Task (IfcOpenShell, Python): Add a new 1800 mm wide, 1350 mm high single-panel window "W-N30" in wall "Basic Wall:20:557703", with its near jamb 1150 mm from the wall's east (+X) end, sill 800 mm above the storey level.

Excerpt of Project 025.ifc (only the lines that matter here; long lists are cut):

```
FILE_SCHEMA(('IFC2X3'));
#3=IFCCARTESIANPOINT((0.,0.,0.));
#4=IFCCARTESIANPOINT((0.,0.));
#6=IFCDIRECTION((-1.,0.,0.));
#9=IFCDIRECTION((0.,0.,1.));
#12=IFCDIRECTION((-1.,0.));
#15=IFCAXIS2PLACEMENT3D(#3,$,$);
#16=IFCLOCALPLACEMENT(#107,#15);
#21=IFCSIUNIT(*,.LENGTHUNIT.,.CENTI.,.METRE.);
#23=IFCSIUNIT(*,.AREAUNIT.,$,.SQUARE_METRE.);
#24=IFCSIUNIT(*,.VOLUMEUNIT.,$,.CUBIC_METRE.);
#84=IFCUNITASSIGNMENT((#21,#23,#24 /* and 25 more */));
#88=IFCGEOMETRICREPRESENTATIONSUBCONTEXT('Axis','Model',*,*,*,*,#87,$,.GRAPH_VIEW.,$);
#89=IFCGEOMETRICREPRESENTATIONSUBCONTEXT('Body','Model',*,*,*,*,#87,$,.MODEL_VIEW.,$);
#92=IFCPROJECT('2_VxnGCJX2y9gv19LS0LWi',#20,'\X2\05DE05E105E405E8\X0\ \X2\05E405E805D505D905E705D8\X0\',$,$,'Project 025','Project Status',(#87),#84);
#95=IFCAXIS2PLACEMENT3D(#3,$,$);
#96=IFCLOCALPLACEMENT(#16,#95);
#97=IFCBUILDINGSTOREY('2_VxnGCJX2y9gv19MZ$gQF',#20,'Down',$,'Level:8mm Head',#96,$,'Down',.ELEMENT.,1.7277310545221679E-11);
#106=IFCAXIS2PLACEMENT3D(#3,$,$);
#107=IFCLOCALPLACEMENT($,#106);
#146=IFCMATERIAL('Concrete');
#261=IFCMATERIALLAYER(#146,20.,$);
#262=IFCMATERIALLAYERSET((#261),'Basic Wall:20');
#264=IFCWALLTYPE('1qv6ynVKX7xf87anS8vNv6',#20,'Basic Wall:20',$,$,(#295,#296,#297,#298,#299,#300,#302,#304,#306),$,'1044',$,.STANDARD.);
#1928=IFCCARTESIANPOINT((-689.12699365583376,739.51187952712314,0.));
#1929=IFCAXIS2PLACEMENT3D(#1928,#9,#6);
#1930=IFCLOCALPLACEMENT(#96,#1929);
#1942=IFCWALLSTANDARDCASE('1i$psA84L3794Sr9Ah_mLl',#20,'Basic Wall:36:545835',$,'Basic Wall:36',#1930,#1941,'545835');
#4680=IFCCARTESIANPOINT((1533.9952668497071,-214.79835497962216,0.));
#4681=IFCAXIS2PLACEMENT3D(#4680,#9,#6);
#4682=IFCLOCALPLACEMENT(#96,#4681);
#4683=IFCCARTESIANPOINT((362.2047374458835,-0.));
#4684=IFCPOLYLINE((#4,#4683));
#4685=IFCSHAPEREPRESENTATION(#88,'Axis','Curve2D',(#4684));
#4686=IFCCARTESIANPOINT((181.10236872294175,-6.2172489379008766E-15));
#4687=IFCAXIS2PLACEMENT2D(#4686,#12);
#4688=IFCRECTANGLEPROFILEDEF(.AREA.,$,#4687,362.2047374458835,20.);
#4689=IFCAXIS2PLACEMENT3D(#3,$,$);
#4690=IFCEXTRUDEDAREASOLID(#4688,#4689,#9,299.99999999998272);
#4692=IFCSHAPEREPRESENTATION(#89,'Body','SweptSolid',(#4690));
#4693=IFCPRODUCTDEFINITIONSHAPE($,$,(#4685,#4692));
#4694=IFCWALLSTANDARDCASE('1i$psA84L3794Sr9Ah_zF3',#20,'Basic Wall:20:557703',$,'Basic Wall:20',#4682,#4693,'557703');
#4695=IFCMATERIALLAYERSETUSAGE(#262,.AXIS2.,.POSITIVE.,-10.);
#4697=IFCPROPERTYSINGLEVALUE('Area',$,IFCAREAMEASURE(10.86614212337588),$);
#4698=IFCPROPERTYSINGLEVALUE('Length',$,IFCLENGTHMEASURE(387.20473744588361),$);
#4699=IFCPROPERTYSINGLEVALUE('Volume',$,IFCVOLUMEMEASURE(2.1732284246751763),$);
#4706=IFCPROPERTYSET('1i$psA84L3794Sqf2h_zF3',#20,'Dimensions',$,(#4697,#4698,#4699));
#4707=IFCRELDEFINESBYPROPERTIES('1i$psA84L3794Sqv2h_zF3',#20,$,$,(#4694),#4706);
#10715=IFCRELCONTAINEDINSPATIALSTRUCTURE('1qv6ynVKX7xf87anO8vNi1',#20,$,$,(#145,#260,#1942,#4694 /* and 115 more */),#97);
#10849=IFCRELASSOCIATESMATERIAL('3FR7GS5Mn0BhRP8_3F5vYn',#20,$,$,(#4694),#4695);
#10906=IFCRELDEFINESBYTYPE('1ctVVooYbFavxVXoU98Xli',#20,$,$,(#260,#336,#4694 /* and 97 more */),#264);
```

```python
import numpy as np
import ifcopenshell
import ifcopenshell.api.feature
import ifcopenshell.api.geometry
import ifcopenshell.api.pset
import ifcopenshell.api.root
import ifcopenshell.api.spatial
import ifcopenshell.api.type
import ifcopenshell.geom
import ifcopenshell.util.element
import ifcopenshell.util.placement
import ifcopenshell.util.representation
import ifcopenshell.util.shape
import ifcopenshell.util.unit

model = ifcopenshell.open("Project 025.ifc")
unit_scale = ifcopenshell.util.unit.calculate_unit_scale(model)
area_scale = ifcopenshell.util.unit.calculate_unit_scale(model, "AREAUNIT")
volume_scale = ifcopenshell.util.unit.calculate_unit_scale(model, "VOLUMEUNIT")
settings = ifcopenshell.geom.settings()


def volume(element):
    """Net volume in cubic metres, openings subtracted."""
    shape = ifcopenshell.geom.create_shape(settings, element)
    return ifcopenshell.util.shape.get_volume(shape.geometry)


wall = model.by_id(4694)
storey = ifcopenshell.util.element.get_container(wall, ifc_class="IfcBuildingStorey")
context = ifcopenshell.util.representation.get_context(model, "Model", "Body", "MODEL_VIEW")
before = volume(wall)

width, height, from_end, sill = 1.8, 1.35, 1.15, 0.8  # metres

# The wall runs along its own X axis, and the end named is its -X end.
wall_shape = ifcopenshell.geom.create_shape(settings, wall)
x, y, z = ifcopenshell.util.shape.get_vertices(wall_shape.geometry).T
start = x.min() + from_end
face, thickness = float(y.min()), float(y.max() - y.min())
wall_matrix = ifcopenshell.util.placement.get_local_placement(wall.ObjectPlacement)
level = ifcopenshell.util.placement.get_local_placement(storey.ObjectPlacement)[2, 3]


def in_wall(x, y):
    """Placement at x, y metres in the wall's axes, at sill height."""
    matrix = wall_matrix.copy()
    matrix[:, 3] = wall_matrix @ np.array([x / unit_scale, y / unit_scale, 0.0, 1.0])
    matrix[2, 3] = level + sill / unit_scale
    return matrix


# Opening: a box that overshoots both wall faces by 50 mm.
opening = ifcopenshell.api.root.create_entity(model, ifc_class="IfcOpeningElement")
box = ifcopenshell.api.geometry.add_wall_representation(
    model, context=context, length=width, height=height, thickness=thickness + 0.1
)
ifcopenshell.api.geometry.assign_representation(model, product=opening, representation=box)
ifcopenshell.api.geometry.edit_object_placement(model, product=opening, matrix=in_wall(start, face - 0.05), is_si=False)
ifcopenshell.api.feature.add_feature(model, feature=opening, element=wall)

window = ifcopenshell.api.root.create_entity(model, ifc_class="IfcWindow", name="W-N30")
window.OverallWidth, window.OverallHeight = width / unit_scale, height / unit_scale
body = ifcopenshell.api.geometry.add_window_representation(
    model,
    context=context,
    overall_width=window.OverallWidth,
    overall_height=window.OverallHeight,
    partition_type="SINGLE_PANEL",
)
ifcopenshell.api.geometry.assign_representation(model, product=window, representation=body)
ifcopenshell.api.spatial.assign_container(model, products=[window], relating_structure=storey)
fills = ifcopenshell.api.feature.add_filling(model, opening=opening, element=window)
fills.OwnerHistory = window.OwnerHistory  # required in IFC2X3

# IFC2X3 keeps the operation on the window style.
style = ifcopenshell.api.root.create_entity(model, ifc_class="IfcWindowStyle", name="W-N30")
style.OperationType, style.ConstructionType = "SINGLE_PANEL", "NOTDEFINED"
style.ParameterTakesPrecedence = style.Sizeable = False
ifcopenshell.api.type.assign_type(model, related_objects=[window], relating_type=style)

# Centre the window in the wall's thickness.
ifcopenshell.api.geometry.edit_object_placement(model, product=window, matrix=in_wall(start, face), is_si=False)
window_shape = ifcopenshell.geom.create_shape(settings, window)
depth = ifcopenshell.util.shape.get_vertices(window_shape.geometry)[:, 1]
offset = face + thickness / 2 - (depth.min() + depth.max()) / 2
ifcopenshell.api.geometry.edit_object_placement(model, product=window, matrix=in_wall(start, offset), is_si=False)

after = volume(wall)

# Update the wall's stored quantities.
pset = model.by_id(ifcopenshell.util.element.get_pset(wall, "Dimensions", should_inherit=False)["id"])
ifcopenshell.api.pset.edit_pset(model, pset=pset, properties={
    "Area": model.create_entity("IfcAreaMeasure", after / thickness / area_scale),
    "Volume": model.create_entity("IfcVolumeMeasure", after / volume_scale),
})

print(f"wall volume {before:.3f} -> {after:.3f} m3")

model.write("Project 025_v2.ifc")
```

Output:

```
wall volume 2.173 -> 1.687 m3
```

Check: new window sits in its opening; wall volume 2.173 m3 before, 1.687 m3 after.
